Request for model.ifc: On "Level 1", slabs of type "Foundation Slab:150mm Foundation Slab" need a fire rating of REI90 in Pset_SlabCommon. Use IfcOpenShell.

First a look at what the model holds.

```python
import ifcopenshell
import ifcopenshell.util.element

model = ifcopenshell.open("model.ifc")
print(model.schema)
storey = next(s for s in model.by_type("IfcBuildingStorey") if s.Name == "Level 1")
slabs = [e for e in ifcopenshell.util.element.get_decomposition(storey) if e.is_a("IfcSlab")]
seen = {}
for e in slabs:
    element_type = ifcopenshell.util.element.get_type(e)
    key = (element_type.Name if element_type != e and element_type else None, ifcopenshell.util.element.get_pset(e, "Pset_SlabCommon", "FireRating"))
    seen[key] = seen.get(key, 0) + 1
for (name, value), count in sorted(seen.items(), key=str):
    print(count, "x", name, "|", value)
```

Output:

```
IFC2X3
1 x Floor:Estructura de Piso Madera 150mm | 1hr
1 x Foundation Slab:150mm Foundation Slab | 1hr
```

```python
import ifcopenshell
import ifcopenshell.api.pset
import ifcopenshell.util.element

model = ifcopenshell.open("model.ifc")

storey = next(s for s in model.by_type("IfcBuildingStorey") if s.Name == "Level 1")
slabs = [e for e in ifcopenshell.util.element.get_decomposition(storey) if e.is_a("IfcSlab")]

count = 0
for e in slabs:
    element_type = ifcopenshell.util.element.get_type(e)
    if element_type in (None, e) or element_type.Name != "Foundation Slab:150mm Foundation Slab":
        continue
    # add_pset returns the element's existing set when there is one.
    pset = ifcopenshell.api.pset.add_pset(model, product=e, name="Pset_SlabCommon")
    ifcopenshell.api.pset.edit_pset(model, pset=pset, properties={"FireRating": "REI90"})
    count += 1

print(count, "slabs updated")

model.write("model_updated.ifc")
```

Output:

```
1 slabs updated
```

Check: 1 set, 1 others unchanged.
